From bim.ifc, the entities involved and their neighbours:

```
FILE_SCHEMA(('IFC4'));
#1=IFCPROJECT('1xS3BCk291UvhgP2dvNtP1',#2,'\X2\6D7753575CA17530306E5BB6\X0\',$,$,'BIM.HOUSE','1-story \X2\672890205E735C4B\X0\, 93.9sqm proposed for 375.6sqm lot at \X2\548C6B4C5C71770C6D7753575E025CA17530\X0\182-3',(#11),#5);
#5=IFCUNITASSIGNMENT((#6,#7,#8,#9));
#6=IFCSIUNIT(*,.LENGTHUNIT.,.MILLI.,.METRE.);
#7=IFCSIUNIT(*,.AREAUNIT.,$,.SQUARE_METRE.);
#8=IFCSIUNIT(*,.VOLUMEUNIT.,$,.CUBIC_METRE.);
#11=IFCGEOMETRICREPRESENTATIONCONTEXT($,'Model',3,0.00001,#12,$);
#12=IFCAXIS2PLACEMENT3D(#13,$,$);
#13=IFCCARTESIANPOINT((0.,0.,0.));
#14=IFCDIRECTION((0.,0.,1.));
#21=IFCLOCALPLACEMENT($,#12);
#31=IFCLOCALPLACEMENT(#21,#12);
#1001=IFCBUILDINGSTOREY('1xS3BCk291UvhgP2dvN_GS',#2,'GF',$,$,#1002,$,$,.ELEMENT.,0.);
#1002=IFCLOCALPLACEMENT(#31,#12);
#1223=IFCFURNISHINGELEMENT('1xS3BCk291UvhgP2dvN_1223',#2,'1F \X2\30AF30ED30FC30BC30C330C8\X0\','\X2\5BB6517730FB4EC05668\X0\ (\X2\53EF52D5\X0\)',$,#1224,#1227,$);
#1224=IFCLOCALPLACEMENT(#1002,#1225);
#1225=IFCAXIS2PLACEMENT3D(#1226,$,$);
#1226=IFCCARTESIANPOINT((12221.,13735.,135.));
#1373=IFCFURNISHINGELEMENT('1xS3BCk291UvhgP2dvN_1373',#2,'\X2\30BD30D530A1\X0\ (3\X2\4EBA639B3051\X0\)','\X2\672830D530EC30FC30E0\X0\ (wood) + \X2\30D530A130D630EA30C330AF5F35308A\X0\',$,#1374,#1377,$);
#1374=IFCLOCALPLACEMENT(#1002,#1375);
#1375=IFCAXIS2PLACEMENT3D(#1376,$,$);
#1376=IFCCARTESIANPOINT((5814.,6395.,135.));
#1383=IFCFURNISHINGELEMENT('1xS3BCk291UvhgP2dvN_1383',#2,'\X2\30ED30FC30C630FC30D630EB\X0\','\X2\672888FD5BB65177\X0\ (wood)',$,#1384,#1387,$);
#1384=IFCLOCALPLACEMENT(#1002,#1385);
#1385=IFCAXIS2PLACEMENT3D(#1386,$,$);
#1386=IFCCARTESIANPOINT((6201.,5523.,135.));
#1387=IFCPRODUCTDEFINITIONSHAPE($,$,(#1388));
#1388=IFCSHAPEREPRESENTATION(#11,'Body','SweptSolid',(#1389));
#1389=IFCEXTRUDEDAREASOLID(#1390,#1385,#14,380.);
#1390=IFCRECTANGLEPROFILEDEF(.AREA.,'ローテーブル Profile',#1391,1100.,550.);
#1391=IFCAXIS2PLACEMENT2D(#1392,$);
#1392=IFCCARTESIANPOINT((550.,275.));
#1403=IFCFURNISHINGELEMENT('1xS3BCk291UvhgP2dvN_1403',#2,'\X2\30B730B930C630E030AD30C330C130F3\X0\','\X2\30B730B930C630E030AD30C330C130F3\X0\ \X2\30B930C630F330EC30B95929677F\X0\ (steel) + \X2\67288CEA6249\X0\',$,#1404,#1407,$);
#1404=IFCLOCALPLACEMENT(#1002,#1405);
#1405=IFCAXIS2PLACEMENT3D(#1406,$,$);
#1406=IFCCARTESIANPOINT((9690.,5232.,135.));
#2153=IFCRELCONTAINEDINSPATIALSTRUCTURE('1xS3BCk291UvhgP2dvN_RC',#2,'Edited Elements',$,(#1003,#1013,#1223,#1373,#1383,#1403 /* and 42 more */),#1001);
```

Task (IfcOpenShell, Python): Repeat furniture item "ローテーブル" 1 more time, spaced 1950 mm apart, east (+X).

```python
import numpy as np
import ifcopenshell
import ifcopenshell.api.geometry
import ifcopenshell.api.root
import ifcopenshell.util.element
import ifcopenshell.util.placement

model = ifcopenshell.open("bim.ifc")


def reuse_history(source, copy):
    """copy_class also copies each property set's owner history, people and application; keep the originals."""
    for rel in copy.IsDefinedBy:
        if rel.is_a("IfcRelDefinesByProperties") and (history := rel.RelatingPropertyDefinition.OwnerHistory):
            rel.RelatingPropertyDefinition.OwnerHistory = source.OwnerHistory
            ifcopenshell.util.element.remove_deep2(model, history)


source = model.by_guid("1xS3BCk291UvhgP2dvN_1383")
base = ifcopenshell.util.placement.get_local_placement(source.ObjectPlacement)
step = np.array([1.0, 0.0, 0.0]) * 1950.0

for i in range(1, 2):
    copy = ifcopenshell.api.root.copy_class(model, product=source)
    copy.Representation = ifcopenshell.util.element.copy_deep(
        model, source.Representation, exclude=["IfcGeometricRepresentationContext", "IfcRepresentationMap"]
    )
    reuse_history(source, copy)
    matrix = base.copy()
    matrix[:3, 3] += i * step
    print("added at", matrix[:3, 3].round(3) + 0.0)
    ifcopenshell.api.geometry.edit_object_placement(model, product=copy, matrix=matrix, is_si=False)

model.write("bim_edited.ifc")
```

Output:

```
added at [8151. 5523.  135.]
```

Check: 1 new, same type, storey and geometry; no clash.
